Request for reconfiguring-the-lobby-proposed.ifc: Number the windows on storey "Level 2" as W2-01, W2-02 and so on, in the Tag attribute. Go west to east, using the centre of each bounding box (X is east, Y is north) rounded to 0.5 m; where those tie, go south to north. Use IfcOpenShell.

First a look at what the model holds.

```python
import ifcopenshell
import ifcopenshell.util.element
import ifcopenshell.util.placement

model = ifcopenshell.open("reconfiguring-the-lobby-proposed.ifc")
print(model.schema)
storey = next(s for s in model.by_type("IfcBuildingStorey") if s.Name == "Level 2")
windows = [e for e in ifcopenshell.util.element.get_decomposition(storey) if e.is_a("IfcWindow")]
for e in sorted(windows, key=lambda e: e.id()):
    origin = ifcopenshell.util.placement.get_local_placement(e.ObjectPlacement)[:3, 3]
    print(e.id(), e.Tag, e.Name, origin.round(2) + 0.0, sep=" | ")
```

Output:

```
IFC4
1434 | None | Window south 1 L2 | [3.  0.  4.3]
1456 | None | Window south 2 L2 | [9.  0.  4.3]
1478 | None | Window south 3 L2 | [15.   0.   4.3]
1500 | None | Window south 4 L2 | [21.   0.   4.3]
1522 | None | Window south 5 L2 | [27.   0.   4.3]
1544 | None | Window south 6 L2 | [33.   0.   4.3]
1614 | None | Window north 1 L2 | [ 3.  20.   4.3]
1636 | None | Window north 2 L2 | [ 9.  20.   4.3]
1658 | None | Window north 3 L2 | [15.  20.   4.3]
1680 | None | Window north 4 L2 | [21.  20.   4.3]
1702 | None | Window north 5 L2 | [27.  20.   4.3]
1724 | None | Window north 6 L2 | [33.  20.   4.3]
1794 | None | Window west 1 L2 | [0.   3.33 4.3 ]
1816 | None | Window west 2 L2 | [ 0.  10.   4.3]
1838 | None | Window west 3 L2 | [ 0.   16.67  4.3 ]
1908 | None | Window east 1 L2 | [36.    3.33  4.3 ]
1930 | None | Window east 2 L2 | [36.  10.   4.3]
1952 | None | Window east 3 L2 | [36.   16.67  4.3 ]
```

```python
import ifcopenshell
import ifcopenshell.geom
import ifcopenshell.util.element
import ifcopenshell.util.shape

model = ifcopenshell.open("reconfiguring-the-lobby-proposed.ifc")
settings = ifcopenshell.geom.settings()
settings.set("use-world-coords", True)


def centre(element):
    shape = ifcopenshell.geom.create_shape(settings, element)
    return ifcopenshell.util.shape.get_bbox_centroid(shape.geometry)


storey = next(s for s in model.by_type("IfcBuildingStorey") if s.Name == "Level 2")
windows = [e for e in ifcopenshell.util.element.get_decomposition(storey) if e.is_a("IfcWindow")]

# Insertion points can sit at a corner or the storey origin, so sort by the geometry (in metres).
centres = {e: centre(e) for e in windows}
windows.sort(key=lambda e: (round(centres[e][0] / 0.5), centres[e][1]))

for i, e in enumerate(windows, start=1):
    number = f"W2-{i:02d}"
    e.Tag = number
    print(e.id(), number)

model.write("reconfiguring-the-lobby-proposed_rev.ifc")
```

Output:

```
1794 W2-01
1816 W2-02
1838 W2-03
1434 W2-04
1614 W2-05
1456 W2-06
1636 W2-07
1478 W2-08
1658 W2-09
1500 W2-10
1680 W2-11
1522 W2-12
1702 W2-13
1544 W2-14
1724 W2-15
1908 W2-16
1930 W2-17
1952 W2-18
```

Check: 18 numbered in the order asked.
